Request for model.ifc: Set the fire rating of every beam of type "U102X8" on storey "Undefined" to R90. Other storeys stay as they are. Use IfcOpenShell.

First a look at what the model holds.

```python
import ifcopenshell
import ifcopenshell.util.element

model = ifcopenshell.open("model.ifc")
print(model.schema)
storey = next(s for s in model.by_type("IfcBuildingStorey") if s.Name == "Undefined")
beams = [e for e in ifcopenshell.util.element.get_decomposition(storey) if e.is_a("IfcBeam")]
seen = {}
for e in beams:
    element_type = ifcopenshell.util.element.get_type(e)
    key = (element_type.Name if element_type != e and element_type else None, ifcopenshell.util.element.get_pset(e, "Pset_BeamCommon", "FireRating"))
    seen[key] = seen.get(key, 0) + 1
for (name, value), count in sorted(seen.items(), key=str):
    print(count, "x", name, "|", value)
```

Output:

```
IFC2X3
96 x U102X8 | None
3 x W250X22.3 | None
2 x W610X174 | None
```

```python
import ifcopenshell
import ifcopenshell.api.pset
import ifcopenshell.util.element

model = ifcopenshell.open("model.ifc")

storey = next(s for s in model.by_type("IfcBuildingStorey") if s.Name == "Undefined")
beams = [e for e in ifcopenshell.util.element.get_decomposition(storey) if e.is_a("IfcBeam")]

count = 0
for e in beams:
    element_type = ifcopenshell.util.element.get_type(e)
    if element_type in (None, e) or element_type.Name != "U102X8":
        continue
    found = ifcopenshell.util.element.get_pset(e, "Pset_BeamCommon", should_inherit=False)
    if found:
        pset = model.by_id(found["id"])
        if len(ifcopenshell.util.element.get_elements_by_pset(pset)) > 1:
            pset = ifcopenshell.api.pset.unshare_pset(model, products=[e], pset=pset)[0]
    else:
        pset = ifcopenshell.api.pset.add_pset(model, product=e, name="Pset_BeamCommon")
    ifcopenshell.api.pset.edit_pset(model, pset=pset, properties={"FireRating": "R90"})
    count += 1

print(count, "beams updated")

model.write("model-out.ifc")
```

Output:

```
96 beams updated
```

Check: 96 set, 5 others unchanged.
